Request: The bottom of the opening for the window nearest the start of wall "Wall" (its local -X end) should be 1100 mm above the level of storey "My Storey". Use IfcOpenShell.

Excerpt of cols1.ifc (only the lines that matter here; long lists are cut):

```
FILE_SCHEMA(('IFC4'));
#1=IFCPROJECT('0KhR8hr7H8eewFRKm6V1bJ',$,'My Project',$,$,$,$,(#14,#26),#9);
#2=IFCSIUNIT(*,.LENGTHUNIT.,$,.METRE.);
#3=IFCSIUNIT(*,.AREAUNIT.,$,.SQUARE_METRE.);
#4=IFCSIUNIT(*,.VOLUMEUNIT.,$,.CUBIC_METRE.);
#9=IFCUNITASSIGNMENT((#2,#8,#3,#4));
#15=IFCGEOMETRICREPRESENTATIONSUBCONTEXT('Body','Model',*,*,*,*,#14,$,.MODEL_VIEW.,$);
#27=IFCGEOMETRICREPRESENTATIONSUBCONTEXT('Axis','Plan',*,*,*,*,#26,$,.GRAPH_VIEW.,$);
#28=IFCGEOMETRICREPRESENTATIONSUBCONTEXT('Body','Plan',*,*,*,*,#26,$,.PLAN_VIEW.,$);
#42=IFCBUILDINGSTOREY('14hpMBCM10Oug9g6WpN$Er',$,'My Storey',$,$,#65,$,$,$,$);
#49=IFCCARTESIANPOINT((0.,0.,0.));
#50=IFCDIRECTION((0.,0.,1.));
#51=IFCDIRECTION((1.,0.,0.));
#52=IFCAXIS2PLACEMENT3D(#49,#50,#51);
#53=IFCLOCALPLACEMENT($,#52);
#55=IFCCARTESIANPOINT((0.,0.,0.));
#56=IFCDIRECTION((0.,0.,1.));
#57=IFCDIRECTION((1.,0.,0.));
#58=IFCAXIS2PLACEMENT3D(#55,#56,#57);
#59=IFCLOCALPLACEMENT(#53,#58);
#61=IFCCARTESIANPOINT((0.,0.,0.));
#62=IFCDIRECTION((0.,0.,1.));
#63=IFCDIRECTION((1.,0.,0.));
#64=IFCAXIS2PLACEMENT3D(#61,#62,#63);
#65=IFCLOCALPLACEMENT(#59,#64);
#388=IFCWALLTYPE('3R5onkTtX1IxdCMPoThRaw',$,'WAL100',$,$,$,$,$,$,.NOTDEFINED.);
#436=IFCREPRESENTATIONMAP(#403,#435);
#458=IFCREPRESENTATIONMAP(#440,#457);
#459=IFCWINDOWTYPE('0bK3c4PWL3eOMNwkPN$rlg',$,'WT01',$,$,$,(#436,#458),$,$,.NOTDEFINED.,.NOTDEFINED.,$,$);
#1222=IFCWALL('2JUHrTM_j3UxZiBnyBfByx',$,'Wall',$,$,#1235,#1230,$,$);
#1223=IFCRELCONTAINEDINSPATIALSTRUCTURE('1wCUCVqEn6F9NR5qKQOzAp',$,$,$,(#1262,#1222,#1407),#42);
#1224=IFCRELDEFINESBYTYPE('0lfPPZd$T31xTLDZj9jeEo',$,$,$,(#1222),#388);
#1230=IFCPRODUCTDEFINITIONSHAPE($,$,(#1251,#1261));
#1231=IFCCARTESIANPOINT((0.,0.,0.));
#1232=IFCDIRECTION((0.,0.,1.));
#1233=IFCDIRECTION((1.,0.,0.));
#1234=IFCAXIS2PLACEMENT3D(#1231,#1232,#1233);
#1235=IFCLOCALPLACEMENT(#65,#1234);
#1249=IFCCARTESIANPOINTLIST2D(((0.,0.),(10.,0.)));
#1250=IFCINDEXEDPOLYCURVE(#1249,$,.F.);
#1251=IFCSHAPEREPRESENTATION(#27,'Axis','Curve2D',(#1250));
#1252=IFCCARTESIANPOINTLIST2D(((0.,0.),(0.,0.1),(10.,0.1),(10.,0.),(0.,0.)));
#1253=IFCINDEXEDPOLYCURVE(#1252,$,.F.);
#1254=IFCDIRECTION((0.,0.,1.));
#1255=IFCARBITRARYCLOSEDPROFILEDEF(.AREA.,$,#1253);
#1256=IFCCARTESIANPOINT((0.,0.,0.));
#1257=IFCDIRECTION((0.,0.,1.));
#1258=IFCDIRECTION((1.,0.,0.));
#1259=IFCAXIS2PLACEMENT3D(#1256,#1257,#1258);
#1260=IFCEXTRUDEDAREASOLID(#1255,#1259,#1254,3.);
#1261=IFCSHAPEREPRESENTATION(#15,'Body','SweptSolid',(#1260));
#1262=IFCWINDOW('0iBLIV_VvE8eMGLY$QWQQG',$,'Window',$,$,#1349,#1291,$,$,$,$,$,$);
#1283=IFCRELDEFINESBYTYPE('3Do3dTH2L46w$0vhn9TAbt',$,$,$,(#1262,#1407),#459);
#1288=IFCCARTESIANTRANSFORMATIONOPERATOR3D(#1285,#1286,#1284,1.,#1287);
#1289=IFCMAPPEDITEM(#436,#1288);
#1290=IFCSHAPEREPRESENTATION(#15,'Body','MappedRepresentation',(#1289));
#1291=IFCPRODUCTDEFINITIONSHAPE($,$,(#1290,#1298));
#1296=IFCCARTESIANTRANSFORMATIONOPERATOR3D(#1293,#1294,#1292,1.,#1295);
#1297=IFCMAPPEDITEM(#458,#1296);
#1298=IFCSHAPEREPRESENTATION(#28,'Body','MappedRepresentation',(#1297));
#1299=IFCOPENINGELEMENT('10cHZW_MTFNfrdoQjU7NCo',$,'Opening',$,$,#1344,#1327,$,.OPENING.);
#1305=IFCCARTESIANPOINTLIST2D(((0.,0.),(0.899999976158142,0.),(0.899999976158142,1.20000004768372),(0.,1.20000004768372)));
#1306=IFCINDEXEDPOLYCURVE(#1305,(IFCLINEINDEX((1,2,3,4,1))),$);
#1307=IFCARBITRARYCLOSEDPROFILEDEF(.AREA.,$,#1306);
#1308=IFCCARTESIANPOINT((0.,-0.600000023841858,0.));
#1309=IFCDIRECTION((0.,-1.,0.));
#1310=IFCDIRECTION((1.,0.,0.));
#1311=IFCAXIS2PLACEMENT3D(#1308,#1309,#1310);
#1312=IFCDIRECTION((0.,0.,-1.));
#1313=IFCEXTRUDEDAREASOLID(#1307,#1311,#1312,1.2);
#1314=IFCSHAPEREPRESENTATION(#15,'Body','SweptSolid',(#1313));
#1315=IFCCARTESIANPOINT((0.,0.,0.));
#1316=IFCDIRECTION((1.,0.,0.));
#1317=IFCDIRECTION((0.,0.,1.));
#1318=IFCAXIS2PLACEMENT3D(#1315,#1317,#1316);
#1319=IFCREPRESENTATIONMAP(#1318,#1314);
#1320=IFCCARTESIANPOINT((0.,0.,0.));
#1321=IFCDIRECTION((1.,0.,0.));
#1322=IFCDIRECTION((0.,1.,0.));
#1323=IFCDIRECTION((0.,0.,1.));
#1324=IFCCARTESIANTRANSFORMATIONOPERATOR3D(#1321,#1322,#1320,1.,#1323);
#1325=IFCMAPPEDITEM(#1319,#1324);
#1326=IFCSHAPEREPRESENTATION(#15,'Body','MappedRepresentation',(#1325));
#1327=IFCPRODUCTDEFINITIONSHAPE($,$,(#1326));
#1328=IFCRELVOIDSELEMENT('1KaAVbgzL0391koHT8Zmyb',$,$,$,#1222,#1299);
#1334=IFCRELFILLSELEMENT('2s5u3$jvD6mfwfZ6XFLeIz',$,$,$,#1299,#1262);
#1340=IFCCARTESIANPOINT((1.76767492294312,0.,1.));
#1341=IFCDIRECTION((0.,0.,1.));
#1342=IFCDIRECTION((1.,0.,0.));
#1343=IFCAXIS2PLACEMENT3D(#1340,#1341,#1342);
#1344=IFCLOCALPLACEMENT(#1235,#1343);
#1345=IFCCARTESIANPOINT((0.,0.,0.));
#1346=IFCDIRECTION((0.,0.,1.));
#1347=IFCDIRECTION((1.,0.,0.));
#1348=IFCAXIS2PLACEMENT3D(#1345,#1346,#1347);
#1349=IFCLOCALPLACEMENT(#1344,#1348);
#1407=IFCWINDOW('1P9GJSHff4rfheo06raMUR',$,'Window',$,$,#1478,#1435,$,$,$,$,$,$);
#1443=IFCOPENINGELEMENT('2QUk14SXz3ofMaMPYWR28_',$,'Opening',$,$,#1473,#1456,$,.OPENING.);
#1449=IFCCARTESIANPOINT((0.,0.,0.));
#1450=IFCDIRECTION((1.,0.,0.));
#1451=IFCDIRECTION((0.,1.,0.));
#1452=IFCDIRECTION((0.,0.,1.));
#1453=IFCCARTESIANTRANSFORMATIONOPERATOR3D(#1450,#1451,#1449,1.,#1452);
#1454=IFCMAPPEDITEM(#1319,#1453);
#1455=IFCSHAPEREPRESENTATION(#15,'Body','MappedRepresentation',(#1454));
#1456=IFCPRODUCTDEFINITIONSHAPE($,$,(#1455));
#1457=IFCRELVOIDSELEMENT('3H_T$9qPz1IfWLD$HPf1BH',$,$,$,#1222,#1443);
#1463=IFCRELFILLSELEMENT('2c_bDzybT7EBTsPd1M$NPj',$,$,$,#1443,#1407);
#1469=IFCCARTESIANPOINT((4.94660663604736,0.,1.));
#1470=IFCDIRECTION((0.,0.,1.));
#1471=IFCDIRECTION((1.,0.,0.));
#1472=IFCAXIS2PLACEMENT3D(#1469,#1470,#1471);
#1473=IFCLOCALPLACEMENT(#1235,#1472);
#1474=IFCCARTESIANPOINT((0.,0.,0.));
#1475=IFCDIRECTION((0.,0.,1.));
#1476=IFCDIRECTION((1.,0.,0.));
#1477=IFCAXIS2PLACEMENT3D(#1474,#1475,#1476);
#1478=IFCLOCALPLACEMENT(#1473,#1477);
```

```python
import numpy as np
import ifcopenshell
import ifcopenshell.api.geometry
import ifcopenshell.geom
import ifcopenshell.util.element
import ifcopenshell.util.placement
import ifcopenshell.util.shape
import ifcopenshell.util.unit

model = ifcopenshell.open("cols1.ifc")
unit_scale = ifcopenshell.util.unit.calculate_unit_scale(model)

window = model.by_guid("0iBLIV_VvE8eMGLY$QWQQG")
opening = window.FillsVoids[0].RelatingOpeningElement
storey = ifcopenshell.util.element.get_container(window, ifc_class="IfcBuildingStorey")
level = ifcopenshell.util.placement.get_local_placement(storey.ObjectPlacement)[2, 3]

# The opening's origin need not be at the sill, so measure its lowest point.
shape = ifcopenshell.geom.create_shape(ifcopenshell.geom.settings(), opening)
bottom = ifcopenshell.util.shape.get_shape_bottom_elevation(shape, shape.geometry) / unit_scale
dz = level + 1.1 - bottom

shift = np.array([0.0, 0.0, dz])
# The window is placed relative to its opening, so it follows when the opening moves.
matrix = ifcopenshell.util.placement.get_local_placement(opening.ObjectPlacement)
matrix[:3, 3] += shift
ifcopenshell.api.geometry.edit_object_placement(
    model, product=opening, matrix=matrix, is_si=False, should_transform_children=True
)

print(f"moved by {dz * unit_scale:+.3f} m")

model.write("cols1-out.ifc")
```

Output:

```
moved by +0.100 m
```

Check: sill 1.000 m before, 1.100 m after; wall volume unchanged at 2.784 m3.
